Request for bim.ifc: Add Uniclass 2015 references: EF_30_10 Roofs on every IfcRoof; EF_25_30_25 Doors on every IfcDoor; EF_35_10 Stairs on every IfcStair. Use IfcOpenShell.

First a look at what the model holds.

```python
import ifcopenshell

model = ifcopenshell.open("bim.ifc")
print(model.schema)
print("classifications:", [c.Name for c in model.by_type("IfcClassification")])
for ifc_class in ("IfcDoor", "IfcRoof", "IfcStair", "IfcWall", "IfcWindow"):
    print(ifc_class, len(model.by_type(ifc_class)))
```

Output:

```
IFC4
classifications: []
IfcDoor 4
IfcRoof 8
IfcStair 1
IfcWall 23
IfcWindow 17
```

```python
import ifcopenshell
import ifcopenshell.api.classification

model = ifcopenshell.open("bim.ifc")

system = ifcopenshell.api.classification.add_classification(model, classification="Uniclass 2015")

codes = {
    "IfcRoof": ("EF_30_10", "Roofs"),
    "IfcDoor": ("EF_25_30_25", "Doors"),
    "IfcStair": ("EF_35_10", "Stairs"),
}
for ifc_class, (code, name) in codes.items():
    products = model.by_type(ifc_class)
    ifcopenshell.api.classification.add_reference(
        model, products=products, classification=system, identification=code, name=name
    )
    print(code, len(products))

model.write("bim_edited.ifc")
```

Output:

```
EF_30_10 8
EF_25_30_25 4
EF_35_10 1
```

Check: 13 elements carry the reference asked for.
